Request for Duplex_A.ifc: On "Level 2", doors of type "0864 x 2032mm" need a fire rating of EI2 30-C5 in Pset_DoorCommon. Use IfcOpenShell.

First a look at what the model holds.

```python
import ifcopenshell
import ifcopenshell.util.element

model = ifcopenshell.open("Duplex_A.ifc")
print(model.schema)
storey = next(s for s in model.by_type("IfcBuildingStorey") if s.Name == "Level 2")
doors = [e for e in ifcopenshell.util.element.get_decomposition(storey) if e.is_a("IfcDoor")]
seen = {}
for e in doors:
    element_type = ifcopenshell.util.element.get_type(e)
    key = (element_type.Name if element_type != e and element_type else None, ifcopenshell.util.element.get_pset(e, "Pset_DoorCommon", "FireRating"))
    seen[key] = seen.get(key, 0) + 1
for (name, value), count in sorted(seen.items(), key=str):
    print(count, "x", name, "|", value)
```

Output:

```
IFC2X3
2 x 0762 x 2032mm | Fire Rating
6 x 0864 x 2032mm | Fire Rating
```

```python
import ifcopenshell
import ifcopenshell.api.pset
import ifcopenshell.util.element

model = ifcopenshell.open("Duplex_A.ifc")

storey = next(s for s in model.by_type("IfcBuildingStorey") if s.Name == "Level 2")
doors = [e for e in ifcopenshell.util.element.get_decomposition(storey) if e.is_a("IfcDoor")]

count = 0
for e in doors:
    element_type = ifcopenshell.util.element.get_type(e)
    if element_type in (None, e) or element_type.Name != "0864 x 2032mm":
        continue
    # add_pset returns the element's existing set when there is one.
    pset = ifcopenshell.api.pset.add_pset(model, product=e, name="Pset_DoorCommon")
    ifcopenshell.api.pset.edit_pset(model, pset=pset, properties={"FireRating": "EI2 30-C5"})
    count += 1

print(count, "doors updated")

model.write("Duplex_A-out.ifc")
```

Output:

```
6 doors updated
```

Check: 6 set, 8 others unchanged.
